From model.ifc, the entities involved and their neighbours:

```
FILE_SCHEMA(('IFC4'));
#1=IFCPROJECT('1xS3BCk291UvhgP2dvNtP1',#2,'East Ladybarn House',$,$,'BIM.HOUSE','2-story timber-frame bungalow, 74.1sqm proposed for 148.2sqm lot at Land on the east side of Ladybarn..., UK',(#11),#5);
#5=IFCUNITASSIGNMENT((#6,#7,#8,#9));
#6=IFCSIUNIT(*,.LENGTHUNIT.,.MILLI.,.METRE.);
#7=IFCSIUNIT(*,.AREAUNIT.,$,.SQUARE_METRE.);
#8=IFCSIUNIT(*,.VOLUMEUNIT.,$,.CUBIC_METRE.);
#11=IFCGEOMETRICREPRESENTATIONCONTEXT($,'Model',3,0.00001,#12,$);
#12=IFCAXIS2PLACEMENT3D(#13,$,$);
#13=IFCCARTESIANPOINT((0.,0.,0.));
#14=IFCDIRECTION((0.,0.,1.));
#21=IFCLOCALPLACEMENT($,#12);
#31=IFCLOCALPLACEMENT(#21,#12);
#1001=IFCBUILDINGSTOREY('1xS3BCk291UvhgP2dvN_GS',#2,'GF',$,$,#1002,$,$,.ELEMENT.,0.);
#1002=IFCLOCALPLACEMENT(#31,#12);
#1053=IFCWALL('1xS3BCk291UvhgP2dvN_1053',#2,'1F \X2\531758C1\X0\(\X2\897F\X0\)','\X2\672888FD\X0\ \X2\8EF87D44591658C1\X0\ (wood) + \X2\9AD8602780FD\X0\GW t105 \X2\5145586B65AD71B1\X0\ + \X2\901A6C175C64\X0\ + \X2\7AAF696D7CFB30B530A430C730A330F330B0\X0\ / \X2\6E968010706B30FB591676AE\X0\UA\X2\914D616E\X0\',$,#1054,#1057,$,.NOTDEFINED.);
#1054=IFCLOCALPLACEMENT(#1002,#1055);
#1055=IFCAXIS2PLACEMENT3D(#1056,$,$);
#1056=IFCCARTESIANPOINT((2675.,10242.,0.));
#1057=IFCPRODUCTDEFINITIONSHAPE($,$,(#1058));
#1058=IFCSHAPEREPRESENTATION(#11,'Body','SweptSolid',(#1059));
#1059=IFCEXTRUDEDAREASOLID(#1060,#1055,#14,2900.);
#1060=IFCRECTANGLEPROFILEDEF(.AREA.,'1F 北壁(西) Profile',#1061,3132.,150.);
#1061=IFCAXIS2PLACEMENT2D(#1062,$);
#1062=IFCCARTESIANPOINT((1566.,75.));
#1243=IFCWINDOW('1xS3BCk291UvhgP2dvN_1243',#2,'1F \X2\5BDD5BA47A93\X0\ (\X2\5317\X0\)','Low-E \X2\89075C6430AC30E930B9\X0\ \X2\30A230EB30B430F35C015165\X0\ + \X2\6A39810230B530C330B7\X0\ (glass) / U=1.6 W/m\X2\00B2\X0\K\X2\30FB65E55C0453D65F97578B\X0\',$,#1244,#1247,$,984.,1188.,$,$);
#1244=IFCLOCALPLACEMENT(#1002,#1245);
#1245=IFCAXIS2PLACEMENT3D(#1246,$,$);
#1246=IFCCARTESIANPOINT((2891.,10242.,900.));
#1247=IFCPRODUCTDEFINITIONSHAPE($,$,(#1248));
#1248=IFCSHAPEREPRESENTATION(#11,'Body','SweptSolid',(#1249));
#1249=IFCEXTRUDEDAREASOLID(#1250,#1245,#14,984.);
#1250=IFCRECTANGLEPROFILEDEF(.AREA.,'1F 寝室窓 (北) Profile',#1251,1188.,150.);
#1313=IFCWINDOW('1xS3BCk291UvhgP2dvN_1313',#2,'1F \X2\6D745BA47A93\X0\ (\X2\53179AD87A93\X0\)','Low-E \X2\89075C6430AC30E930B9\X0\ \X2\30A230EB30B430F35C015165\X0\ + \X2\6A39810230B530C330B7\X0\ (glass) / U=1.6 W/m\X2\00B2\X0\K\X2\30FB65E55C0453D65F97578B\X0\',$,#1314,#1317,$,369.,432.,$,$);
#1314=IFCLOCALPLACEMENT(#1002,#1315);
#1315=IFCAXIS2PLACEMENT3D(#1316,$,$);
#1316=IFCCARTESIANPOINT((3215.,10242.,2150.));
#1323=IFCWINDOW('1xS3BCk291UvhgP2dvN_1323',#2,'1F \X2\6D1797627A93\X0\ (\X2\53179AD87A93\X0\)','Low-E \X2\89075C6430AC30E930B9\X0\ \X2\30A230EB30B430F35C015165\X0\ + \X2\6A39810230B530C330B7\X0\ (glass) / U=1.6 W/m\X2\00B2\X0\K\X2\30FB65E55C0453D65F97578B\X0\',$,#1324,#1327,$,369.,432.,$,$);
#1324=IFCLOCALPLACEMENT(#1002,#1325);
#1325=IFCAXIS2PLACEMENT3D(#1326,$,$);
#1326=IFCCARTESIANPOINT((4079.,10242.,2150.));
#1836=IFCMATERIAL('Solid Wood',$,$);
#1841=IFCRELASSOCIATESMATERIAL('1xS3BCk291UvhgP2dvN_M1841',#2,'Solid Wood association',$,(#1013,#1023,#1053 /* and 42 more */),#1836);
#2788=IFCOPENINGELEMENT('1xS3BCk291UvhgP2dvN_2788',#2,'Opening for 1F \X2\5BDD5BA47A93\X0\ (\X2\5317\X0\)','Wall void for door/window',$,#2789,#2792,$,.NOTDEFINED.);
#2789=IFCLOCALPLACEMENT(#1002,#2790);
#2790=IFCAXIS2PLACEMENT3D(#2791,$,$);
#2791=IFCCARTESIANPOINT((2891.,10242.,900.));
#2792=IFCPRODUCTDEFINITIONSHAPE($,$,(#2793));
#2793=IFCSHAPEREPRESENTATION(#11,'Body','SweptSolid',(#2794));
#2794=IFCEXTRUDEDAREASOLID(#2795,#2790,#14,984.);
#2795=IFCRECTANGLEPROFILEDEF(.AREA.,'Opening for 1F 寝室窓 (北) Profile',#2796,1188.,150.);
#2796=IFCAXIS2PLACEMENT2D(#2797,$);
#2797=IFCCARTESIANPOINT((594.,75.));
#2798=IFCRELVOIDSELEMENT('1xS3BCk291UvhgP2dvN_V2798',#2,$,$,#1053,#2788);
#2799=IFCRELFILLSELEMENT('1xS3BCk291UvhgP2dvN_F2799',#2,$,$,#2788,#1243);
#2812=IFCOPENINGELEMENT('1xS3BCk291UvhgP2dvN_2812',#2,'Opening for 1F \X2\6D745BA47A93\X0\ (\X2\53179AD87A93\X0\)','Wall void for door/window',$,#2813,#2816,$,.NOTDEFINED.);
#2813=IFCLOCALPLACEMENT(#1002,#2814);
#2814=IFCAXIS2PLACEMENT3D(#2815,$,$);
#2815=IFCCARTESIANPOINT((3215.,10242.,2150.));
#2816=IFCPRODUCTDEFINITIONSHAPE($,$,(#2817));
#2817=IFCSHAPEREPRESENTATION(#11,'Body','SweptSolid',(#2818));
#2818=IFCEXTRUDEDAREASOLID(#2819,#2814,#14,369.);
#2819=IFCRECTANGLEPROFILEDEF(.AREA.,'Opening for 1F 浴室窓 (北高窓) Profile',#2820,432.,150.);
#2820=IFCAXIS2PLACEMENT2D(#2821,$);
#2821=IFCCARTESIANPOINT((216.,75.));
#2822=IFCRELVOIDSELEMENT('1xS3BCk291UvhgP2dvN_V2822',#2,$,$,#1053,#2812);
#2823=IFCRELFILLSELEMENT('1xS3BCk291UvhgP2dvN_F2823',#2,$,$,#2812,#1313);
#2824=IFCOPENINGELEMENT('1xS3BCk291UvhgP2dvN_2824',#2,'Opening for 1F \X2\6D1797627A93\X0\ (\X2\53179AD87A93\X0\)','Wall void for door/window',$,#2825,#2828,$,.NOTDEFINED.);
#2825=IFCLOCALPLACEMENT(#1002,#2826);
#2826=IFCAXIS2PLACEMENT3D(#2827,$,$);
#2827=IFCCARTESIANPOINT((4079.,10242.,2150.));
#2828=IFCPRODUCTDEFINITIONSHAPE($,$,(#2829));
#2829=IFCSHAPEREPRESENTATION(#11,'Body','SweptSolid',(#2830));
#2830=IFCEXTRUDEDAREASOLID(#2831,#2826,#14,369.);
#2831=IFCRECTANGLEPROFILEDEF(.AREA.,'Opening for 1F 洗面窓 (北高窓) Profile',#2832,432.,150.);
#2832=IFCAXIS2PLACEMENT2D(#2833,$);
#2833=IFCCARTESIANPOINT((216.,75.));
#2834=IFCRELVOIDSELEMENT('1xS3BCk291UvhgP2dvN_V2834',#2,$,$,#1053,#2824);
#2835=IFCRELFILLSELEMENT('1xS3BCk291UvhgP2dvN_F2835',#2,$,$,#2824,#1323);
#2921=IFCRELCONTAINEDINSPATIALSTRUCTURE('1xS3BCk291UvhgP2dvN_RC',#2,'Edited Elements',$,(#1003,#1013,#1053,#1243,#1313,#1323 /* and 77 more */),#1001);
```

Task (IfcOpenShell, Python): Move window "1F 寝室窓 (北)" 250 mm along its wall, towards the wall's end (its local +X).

```python
import ifcopenshell
import ifcopenshell.api.geometry
import ifcopenshell.util.placement

model = ifcopenshell.open("model.ifc")

window = model.by_guid("1xS3BCk291UvhgP2dvN_1243")
opening = window.FillsVoids[0].RelatingOpeningElement
wall = opening.VoidsElements[0].RelatingBuildingElement

wall_matrix = ifcopenshell.util.placement.get_local_placement(wall.ObjectPlacement)
shift = wall_matrix[:3, 0] * 250.0
before = ifcopenshell.util.placement.get_local_placement(window.ObjectPlacement)[:3, 3].copy()

# The window is not placed relative to its opening, so move both.
for product in (opening, window):
    matrix = ifcopenshell.util.placement.get_local_placement(product.ObjectPlacement)
    matrix[:3, 3] += shift
    ifcopenshell.api.geometry.edit_object_placement(model, product=product, matrix=matrix, is_si=False)

after = ifcopenshell.util.placement.get_local_placement(window.ObjectPlacement)[:3, 3]
print("window moved by", (after - before).round(3) + 0.0)

model.write("model_v2.ifc")
```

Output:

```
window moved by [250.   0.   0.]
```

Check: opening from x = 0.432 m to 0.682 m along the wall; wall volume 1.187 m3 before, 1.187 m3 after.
